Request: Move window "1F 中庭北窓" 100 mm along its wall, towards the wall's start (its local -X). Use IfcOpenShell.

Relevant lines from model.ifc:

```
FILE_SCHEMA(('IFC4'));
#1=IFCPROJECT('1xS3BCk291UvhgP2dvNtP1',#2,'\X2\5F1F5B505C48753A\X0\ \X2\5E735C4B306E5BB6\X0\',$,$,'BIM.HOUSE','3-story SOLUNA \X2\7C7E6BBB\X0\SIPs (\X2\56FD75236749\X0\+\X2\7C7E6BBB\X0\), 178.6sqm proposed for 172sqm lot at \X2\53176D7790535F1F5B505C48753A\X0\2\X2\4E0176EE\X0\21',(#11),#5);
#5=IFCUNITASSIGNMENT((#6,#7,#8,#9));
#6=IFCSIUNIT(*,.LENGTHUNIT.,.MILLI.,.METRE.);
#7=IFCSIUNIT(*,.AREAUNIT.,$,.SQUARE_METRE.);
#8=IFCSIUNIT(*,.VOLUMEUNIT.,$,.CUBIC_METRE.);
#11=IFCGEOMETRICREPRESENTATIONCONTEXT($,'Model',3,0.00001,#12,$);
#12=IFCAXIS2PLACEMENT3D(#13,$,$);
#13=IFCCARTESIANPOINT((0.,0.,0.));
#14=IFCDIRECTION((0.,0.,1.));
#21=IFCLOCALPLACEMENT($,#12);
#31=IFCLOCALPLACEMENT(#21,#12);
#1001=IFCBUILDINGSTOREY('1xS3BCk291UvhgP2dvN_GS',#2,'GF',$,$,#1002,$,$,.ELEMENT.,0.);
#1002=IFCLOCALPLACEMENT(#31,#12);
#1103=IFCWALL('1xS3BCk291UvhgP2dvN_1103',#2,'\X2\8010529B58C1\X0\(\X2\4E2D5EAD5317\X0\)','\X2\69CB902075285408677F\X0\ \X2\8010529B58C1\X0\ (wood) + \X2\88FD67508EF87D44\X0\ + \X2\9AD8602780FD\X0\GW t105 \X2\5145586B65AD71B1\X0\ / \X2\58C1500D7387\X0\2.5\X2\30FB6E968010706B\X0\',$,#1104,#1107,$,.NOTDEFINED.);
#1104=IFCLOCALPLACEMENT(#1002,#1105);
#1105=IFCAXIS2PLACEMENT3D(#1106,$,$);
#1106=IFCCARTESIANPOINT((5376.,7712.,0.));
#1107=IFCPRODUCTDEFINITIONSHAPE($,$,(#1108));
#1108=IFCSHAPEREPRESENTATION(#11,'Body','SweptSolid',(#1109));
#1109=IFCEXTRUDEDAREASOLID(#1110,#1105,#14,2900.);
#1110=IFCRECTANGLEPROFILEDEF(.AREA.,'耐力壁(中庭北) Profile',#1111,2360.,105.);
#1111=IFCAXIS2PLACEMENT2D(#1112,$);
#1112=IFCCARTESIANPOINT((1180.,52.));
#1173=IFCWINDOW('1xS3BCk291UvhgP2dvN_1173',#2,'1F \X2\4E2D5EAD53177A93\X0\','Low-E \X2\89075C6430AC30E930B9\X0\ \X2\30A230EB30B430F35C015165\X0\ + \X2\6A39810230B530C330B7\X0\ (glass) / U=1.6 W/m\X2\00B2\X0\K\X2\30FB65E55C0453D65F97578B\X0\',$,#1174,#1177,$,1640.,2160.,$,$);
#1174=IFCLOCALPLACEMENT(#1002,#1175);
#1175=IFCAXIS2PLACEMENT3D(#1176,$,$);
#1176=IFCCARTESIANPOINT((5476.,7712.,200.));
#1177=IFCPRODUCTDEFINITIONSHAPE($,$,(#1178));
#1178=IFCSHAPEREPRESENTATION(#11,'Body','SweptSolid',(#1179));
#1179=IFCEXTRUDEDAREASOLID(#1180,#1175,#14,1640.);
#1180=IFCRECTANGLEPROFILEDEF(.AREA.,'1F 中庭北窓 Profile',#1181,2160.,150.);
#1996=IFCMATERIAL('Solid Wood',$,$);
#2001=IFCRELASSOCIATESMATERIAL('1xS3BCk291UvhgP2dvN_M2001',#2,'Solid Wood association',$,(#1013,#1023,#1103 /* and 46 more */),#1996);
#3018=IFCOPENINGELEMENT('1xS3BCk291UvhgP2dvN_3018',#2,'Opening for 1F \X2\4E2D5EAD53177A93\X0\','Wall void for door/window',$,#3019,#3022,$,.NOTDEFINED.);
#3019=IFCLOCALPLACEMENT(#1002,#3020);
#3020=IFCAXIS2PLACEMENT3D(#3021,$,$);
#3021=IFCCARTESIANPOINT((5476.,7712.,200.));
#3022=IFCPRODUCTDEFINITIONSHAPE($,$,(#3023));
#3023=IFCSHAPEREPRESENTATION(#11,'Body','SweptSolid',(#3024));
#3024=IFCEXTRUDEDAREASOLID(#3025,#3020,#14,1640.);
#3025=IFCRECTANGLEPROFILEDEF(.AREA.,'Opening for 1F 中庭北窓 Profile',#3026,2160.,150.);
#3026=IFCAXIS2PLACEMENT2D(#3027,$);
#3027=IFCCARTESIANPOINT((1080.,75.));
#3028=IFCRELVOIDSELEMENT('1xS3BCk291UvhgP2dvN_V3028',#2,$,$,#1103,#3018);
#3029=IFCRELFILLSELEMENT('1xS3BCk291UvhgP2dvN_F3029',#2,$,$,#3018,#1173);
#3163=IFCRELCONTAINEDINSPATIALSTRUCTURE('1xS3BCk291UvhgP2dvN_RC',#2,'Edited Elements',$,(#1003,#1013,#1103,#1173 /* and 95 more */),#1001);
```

```python
import ifcopenshell
import ifcopenshell.api.geometry
import ifcopenshell.util.placement
import ifcopenshell.util.unit

model = ifcopenshell.open("model.ifc")
unit_scale = ifcopenshell.util.unit.calculate_unit_scale(model)

window = model.by_guid("1xS3BCk291UvhgP2dvN_1173")
opening = window.FillsVoids[0].RelatingOpeningElement
wall = opening.VoidsElements[0].RelatingBuildingElement

wall_matrix = ifcopenshell.util.placement.get_local_placement(wall.ObjectPlacement)
shift = wall_matrix[:3, 0] * -0.1 / unit_scale
before = ifcopenshell.util.placement.get_local_placement(window.ObjectPlacement)[:3, 3].copy()

# The window is not placed relative to its opening, so move both.
for product in (opening, window):
    matrix = ifcopenshell.util.placement.get_local_placement(product.ObjectPlacement)
    matrix[:3, 3] += shift
    ifcopenshell.api.geometry.edit_object_placement(model, product=product, matrix=matrix, is_si=False)

after = ifcopenshell.util.placement.get_local_placement(window.ObjectPlacement)[:3, 3]
print("window moved by", (after - before).round(3) + 0.0)

model.write("model_v2.ifc")
```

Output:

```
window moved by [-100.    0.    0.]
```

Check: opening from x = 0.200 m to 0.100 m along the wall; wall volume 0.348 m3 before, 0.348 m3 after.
